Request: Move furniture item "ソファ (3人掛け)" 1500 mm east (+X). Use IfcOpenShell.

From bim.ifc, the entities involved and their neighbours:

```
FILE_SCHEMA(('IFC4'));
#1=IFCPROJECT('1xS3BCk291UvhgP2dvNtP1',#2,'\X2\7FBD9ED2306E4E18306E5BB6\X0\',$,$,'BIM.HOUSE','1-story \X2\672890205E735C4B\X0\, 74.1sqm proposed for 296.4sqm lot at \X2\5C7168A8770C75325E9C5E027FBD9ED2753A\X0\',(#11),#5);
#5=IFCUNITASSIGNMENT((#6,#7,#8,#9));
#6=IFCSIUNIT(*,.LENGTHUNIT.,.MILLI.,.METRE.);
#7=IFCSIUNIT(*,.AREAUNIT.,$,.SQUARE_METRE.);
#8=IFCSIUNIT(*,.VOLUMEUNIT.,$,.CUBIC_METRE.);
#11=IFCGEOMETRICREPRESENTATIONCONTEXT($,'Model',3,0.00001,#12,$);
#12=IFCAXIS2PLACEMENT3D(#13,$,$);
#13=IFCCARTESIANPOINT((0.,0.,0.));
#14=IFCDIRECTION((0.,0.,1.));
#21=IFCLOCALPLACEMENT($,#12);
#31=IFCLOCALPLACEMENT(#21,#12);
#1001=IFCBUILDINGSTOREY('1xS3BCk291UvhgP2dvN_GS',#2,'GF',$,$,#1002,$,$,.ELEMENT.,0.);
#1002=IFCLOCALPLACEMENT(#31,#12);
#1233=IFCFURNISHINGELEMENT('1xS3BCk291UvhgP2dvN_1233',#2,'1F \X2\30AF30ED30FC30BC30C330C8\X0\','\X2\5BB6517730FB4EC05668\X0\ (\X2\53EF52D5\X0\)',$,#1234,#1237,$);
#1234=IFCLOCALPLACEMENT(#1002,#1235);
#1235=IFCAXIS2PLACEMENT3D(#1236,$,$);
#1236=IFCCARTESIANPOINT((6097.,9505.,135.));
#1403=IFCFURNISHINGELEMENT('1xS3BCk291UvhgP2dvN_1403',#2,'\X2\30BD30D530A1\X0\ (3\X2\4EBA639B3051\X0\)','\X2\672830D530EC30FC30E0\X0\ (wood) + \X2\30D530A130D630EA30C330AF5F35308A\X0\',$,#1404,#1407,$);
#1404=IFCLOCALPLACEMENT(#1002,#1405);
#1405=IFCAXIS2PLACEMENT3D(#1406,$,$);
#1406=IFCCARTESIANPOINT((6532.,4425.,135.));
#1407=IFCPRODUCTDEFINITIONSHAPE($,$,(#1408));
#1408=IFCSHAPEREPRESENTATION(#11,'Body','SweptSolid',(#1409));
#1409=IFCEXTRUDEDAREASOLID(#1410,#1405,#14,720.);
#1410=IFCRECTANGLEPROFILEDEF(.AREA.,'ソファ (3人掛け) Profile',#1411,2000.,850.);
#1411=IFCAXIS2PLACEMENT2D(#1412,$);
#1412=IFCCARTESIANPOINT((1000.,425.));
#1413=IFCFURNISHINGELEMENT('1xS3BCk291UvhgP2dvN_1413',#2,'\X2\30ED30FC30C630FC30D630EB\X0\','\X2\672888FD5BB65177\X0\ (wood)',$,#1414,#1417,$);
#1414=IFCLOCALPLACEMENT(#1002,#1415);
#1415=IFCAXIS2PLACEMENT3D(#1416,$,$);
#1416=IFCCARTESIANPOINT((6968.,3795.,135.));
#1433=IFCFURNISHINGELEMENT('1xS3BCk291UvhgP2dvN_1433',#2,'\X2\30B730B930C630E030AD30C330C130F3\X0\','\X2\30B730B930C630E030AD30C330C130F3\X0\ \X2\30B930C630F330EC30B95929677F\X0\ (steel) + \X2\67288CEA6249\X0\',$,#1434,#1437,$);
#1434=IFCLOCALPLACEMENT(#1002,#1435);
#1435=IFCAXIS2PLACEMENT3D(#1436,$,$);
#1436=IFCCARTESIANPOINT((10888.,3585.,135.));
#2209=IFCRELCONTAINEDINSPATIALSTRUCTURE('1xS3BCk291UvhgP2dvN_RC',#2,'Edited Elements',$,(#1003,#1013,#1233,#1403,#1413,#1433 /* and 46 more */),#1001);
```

```python
import ifcopenshell
import ifcopenshell.api.geometry
import ifcopenshell.util.placement
import ifcopenshell.util.unit

model = ifcopenshell.open("bim.ifc")
unit_scale = ifcopenshell.util.unit.calculate_unit_scale(model)

item = model.by_id(1403)
matrix = ifcopenshell.util.placement.get_local_placement(item.ObjectPlacement)
matrix[0, 3] += 1.5 / unit_scale
ifcopenshell.api.geometry.edit_object_placement(model, product=item, matrix=matrix, is_si=False)

print(ifcopenshell.util.placement.get_local_placement(item.ObjectPlacement).round(3) + 0.0)

model.write("bim_updated.ifc")
```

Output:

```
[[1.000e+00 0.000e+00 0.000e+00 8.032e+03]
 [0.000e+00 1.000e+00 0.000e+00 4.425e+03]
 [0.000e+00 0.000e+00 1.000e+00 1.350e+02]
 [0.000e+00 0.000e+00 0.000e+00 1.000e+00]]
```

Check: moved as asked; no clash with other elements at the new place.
